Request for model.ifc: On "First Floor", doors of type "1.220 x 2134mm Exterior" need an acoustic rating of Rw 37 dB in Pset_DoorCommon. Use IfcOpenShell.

First a look at what the model holds.

```python
import ifcopenshell
import ifcopenshell.util.element

model = ifcopenshell.open("model.ifc")
print(model.schema)
storey = next(s for s in model.by_type("IfcBuildingStorey") if s.Name == "First Floor")
doors = [e for e in ifcopenshell.util.element.get_decomposition(storey) if e.is_a("IfcDoor")]
seen = {}
for e in doors:
    element_type = ifcopenshell.util.element.get_type(e)
    key = (element_type.Name if element_type != e and element_type else None, ifcopenshell.util.element.get_pset(e, "Pset_DoorCommon", "AcousticRating"))
    seen[key] = seen.get(key, 0) + 1
for (name, value), count in sorted(seen.items(), key=str):
    print(count, "x", name, "|", value)
```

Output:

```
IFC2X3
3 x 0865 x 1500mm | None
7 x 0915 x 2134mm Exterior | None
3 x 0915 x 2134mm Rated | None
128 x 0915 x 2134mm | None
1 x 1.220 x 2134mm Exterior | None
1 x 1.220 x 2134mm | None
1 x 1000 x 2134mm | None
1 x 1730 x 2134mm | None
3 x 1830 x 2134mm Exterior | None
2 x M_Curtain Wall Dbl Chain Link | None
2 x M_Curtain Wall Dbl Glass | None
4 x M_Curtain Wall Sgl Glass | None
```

```python
import ifcopenshell
import ifcopenshell.api.pset
import ifcopenshell.util.element

model = ifcopenshell.open("model.ifc")

storey = next(s for s in model.by_type("IfcBuildingStorey") if s.Name == "First Floor")
doors = [e for e in ifcopenshell.util.element.get_decomposition(storey) if e.is_a("IfcDoor")]

count = 0
for e in doors:
    element_type = ifcopenshell.util.element.get_type(e)
    if element_type in (None, e) or element_type.Name != "1.220 x 2134mm Exterior":
        continue
    # add_pset returns the element's existing set when there is one.
    pset = ifcopenshell.api.pset.add_pset(model, product=e, name="Pset_DoorCommon")
    ifcopenshell.api.pset.edit_pset(model, pset=pset, properties={"AcousticRating": "Rw 37 dB"})
    count += 1

print(count, "doors updated")

model.write("model_updated.ifc")
```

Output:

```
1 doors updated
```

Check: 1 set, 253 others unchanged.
